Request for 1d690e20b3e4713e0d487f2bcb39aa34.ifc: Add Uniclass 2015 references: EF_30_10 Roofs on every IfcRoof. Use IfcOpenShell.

First a look at what the model holds.

```python
import ifcopenshell

model = ifcopenshell.open("1d690e20b3e4713e0d487f2bcb39aa34.ifc")
print(model.schema)
print("classifications:", [c.Name for c in model.by_type("IfcClassification")])
for ifc_class in ("IfcDoor", "IfcRoof", "IfcStair", "IfcWall", "IfcWindow"):
    print(ifc_class, len(model.by_type(ifc_class)))
```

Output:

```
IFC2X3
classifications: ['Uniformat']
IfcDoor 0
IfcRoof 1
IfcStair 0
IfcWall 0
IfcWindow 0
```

```python
import ifcopenshell
import ifcopenshell.api.classification

model = ifcopenshell.open("1d690e20b3e4713e0d487f2bcb39aa34.ifc")

# IFC2X3 requires Source and Edition and has no link from the project to the system.
system = model.create_entity("IfcClassification", Source="NBS", Edition="2015", Name="Uniclass 2015")

codes = {
    "IfcRoof": ("EF_30_10", "Roofs"),
}
for ifc_class, (code, name) in codes.items():
    products = model.by_type(ifc_class)
    ifcopenshell.api.classification.add_reference(
        model, products=products, classification=system, identification=code, name=name
    )
    print(code, len(products))

model.write("1d690e20b3e4713e0d487f2bcb39aa34_edited.ifc")
```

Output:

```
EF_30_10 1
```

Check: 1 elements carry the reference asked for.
